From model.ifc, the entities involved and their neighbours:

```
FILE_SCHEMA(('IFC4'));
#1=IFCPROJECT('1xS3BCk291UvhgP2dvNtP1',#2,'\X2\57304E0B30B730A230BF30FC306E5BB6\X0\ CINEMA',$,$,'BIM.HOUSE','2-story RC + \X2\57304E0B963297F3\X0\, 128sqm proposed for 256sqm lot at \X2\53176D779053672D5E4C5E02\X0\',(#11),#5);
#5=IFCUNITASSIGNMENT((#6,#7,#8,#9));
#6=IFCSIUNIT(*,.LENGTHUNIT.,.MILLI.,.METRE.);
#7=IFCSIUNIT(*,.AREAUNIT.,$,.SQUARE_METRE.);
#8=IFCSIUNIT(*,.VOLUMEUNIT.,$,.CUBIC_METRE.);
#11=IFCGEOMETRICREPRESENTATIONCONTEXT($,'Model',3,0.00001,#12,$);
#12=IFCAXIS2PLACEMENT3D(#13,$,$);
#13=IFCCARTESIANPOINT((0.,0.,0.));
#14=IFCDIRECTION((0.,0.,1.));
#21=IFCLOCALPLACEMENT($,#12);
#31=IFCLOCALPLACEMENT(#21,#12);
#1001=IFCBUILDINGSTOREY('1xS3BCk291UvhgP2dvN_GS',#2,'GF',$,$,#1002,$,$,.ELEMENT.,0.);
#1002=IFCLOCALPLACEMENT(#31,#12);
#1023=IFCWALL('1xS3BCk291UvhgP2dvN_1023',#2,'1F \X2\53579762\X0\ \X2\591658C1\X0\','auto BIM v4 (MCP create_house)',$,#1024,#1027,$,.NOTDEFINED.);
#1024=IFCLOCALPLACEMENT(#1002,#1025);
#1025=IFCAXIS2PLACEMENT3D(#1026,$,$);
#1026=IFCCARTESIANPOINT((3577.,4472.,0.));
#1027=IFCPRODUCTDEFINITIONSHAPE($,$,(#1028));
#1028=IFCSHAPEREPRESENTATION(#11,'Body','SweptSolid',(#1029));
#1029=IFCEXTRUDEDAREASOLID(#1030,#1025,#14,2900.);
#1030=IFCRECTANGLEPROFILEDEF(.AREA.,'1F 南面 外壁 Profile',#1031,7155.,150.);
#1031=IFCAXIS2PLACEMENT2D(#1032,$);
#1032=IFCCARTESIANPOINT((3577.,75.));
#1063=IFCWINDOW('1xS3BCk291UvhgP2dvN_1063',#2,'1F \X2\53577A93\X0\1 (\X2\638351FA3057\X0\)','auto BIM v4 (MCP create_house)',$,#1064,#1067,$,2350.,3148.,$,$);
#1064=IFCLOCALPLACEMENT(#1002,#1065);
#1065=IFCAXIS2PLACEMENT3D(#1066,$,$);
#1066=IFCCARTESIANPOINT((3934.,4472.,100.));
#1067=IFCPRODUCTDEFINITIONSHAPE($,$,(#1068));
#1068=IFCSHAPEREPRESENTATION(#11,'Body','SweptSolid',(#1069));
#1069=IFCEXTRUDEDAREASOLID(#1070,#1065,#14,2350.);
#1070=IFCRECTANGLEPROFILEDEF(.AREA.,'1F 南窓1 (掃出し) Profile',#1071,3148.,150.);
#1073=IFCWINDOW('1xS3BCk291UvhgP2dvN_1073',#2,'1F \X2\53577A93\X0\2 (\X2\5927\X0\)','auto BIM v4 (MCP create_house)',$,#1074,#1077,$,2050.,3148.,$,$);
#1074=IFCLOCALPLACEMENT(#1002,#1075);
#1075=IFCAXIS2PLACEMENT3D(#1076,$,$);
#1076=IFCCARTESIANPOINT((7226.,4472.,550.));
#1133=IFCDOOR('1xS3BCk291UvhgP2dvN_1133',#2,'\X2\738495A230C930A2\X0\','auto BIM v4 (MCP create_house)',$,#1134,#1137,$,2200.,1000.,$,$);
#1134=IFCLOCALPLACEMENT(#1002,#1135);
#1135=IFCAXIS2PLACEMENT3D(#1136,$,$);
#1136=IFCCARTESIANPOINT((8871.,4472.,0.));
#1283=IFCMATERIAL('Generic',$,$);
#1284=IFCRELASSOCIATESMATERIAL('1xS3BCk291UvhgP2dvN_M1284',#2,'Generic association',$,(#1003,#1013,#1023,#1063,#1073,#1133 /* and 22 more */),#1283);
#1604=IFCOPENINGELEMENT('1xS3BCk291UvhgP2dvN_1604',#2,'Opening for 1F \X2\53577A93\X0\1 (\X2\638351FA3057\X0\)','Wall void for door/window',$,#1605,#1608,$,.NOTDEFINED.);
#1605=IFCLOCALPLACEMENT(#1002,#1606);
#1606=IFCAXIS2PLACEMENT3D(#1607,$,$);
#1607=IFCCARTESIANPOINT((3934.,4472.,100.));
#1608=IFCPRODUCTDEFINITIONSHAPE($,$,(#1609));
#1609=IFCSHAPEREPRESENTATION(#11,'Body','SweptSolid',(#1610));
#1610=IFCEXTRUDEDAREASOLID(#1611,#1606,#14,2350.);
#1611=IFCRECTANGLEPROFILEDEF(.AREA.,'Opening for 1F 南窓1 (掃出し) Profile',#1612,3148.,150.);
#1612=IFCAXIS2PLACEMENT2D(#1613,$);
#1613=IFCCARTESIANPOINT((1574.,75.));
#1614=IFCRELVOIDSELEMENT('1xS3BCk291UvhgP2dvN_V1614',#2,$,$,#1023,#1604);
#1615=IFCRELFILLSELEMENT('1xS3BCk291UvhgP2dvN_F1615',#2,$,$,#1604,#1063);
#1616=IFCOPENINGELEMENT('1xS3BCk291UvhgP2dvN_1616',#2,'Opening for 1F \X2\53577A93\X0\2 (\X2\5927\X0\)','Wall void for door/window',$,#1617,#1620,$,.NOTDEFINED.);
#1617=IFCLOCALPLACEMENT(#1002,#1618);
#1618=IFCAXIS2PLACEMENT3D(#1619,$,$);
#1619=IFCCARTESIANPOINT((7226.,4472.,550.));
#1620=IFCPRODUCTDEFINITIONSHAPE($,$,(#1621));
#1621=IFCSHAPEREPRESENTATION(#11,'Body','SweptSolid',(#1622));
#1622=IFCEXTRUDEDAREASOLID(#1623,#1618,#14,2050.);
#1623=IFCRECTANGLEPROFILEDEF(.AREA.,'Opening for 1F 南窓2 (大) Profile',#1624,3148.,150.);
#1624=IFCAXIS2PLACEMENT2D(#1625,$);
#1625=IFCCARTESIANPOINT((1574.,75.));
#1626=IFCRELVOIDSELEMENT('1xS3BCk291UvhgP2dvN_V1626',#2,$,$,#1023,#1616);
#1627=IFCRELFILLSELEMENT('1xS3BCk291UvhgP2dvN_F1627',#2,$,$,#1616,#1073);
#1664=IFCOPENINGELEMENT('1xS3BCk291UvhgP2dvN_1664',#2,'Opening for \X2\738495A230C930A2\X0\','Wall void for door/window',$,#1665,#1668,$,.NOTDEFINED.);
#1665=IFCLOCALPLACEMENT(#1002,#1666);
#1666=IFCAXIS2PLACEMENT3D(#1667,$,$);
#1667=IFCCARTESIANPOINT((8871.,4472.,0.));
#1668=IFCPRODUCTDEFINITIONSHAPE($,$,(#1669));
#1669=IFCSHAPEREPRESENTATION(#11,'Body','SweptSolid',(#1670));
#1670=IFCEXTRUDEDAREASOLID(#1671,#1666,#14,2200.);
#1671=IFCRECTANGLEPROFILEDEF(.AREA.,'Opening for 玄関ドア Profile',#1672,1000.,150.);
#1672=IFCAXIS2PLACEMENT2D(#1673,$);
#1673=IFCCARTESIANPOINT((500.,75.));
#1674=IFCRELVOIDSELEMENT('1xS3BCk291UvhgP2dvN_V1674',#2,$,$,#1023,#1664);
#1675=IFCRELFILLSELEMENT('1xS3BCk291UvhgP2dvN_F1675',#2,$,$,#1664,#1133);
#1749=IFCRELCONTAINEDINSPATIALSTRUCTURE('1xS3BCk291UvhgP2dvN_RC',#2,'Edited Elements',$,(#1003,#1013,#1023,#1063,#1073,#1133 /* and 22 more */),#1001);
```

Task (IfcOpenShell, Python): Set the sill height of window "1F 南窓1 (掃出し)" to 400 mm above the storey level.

```python
import numpy as np
import ifcopenshell
import ifcopenshell.api.geometry
import ifcopenshell.geom
import ifcopenshell.util.element
import ifcopenshell.util.placement
import ifcopenshell.util.shape
import ifcopenshell.util.unit

model = ifcopenshell.open("model.ifc")
unit_scale = ifcopenshell.util.unit.calculate_unit_scale(model)

window = model.by_guid("1xS3BCk291UvhgP2dvN_1063")
opening = window.FillsVoids[0].RelatingOpeningElement
storey = ifcopenshell.util.element.get_container(window, ifc_class="IfcBuildingStorey")
level = ifcopenshell.util.placement.get_local_placement(storey.ObjectPlacement)[2, 3]

# The opening's origin need not be at the sill, so measure its lowest point.
shape = ifcopenshell.geom.create_shape(ifcopenshell.geom.settings(), opening)
bottom = ifcopenshell.util.shape.get_shape_bottom_elevation(shape, shape.geometry) / unit_scale
dz = level + 0.4 / unit_scale - bottom

shift = np.array([0.0, 0.0, dz])
# The window is not placed relative to its opening, so move both.
for product in (opening, window):
    matrix = ifcopenshell.util.placement.get_local_placement(product.ObjectPlacement)
    matrix[:3, 3] += shift
    ifcopenshell.api.geometry.edit_object_placement(model, product=product, matrix=matrix, is_si=False)

print(f"moved by {dz * unit_scale:+.3f} m")

model.write("model_updated.ifc")
```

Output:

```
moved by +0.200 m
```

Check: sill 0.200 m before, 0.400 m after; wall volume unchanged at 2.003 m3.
